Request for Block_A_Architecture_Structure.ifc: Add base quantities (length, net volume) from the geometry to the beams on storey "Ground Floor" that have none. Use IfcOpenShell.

First a look at what the model holds.

```python
import ifcopenshell
import ifcopenshell.util.element
import ifcopenshell.util.unit

model = ifcopenshell.open("Block_A_Architecture_Structure.ifc")
print(model.schema)
for unit_type in ("LENGTHUNIT", "AREAUNIT", "VOLUMEUNIT"):
    print(unit_type, ifcopenshell.util.unit.calculate_unit_scale(model, unit_type))
storey = next(s for s in model.by_type("IfcBuildingStorey") if s.Name == "Ground Floor")
beams = [e for e in ifcopenshell.util.element.get_decomposition(storey) if e.is_a("IfcBeam")]
for e in sorted(beams, key=lambda e: e.id()):
    print(e.id(), e.is_a(), e.Name, list(ifcopenshell.util.element.get_psets(e, qtos_only=True)), sep=" | ")
```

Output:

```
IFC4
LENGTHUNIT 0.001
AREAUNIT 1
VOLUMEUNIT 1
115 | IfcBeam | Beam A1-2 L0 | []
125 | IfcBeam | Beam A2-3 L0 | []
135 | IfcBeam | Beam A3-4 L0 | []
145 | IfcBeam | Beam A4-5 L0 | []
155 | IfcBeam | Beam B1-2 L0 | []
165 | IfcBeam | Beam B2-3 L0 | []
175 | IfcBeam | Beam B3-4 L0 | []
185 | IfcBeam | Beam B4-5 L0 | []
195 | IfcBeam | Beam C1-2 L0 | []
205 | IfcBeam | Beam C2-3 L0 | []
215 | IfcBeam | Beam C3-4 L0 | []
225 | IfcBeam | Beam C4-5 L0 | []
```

```python
import ifcopenshell
import ifcopenshell.api.pset
import ifcopenshell.geom
import ifcopenshell.util.element
import ifcopenshell.util.shape
import ifcopenshell.util.unit

model = ifcopenshell.open("Block_A_Architecture_Structure.ifc")
unit_scale = ifcopenshell.util.unit.calculate_unit_scale(model)
volume_scale = ifcopenshell.util.unit.calculate_unit_scale(model, "VOLUMEUNIT")
settings = ifcopenshell.geom.settings()

storey = next(s for s in model.by_type("IfcBuildingStorey") if s.Name == "Ground Floor")
beams = [e for e in ifcopenshell.util.element.get_decomposition(storey) if e.is_a("IfcBeam")]

for e in sorted(beams, key=lambda e: e.id()):
    if ifcopenshell.util.element.get_psets(e, qtos_only=True, should_inherit=False):
        continue
    # Geometry comes back in metres, in the element's own axes.
    shape = ifcopenshell.geom.create_shape(settings, e)
    values = {
        "Length": ifcopenshell.util.shape.get_max_xyz(shape.geometry) / unit_scale,
        "NetVolume": ifcopenshell.util.shape.get_volume(shape.geometry) / volume_scale,
    }
    qto = ifcopenshell.api.pset.add_qto(model, product=e, name="Qto_BeamBaseQuantities")
    ifcopenshell.api.pset.edit_qto(model, qto=qto, properties=values)
    print(e.id(), {k: round(v, 3) for k, v in values.items()})

model.write("Block_A_Architecture_Structure_rev.ifc")
```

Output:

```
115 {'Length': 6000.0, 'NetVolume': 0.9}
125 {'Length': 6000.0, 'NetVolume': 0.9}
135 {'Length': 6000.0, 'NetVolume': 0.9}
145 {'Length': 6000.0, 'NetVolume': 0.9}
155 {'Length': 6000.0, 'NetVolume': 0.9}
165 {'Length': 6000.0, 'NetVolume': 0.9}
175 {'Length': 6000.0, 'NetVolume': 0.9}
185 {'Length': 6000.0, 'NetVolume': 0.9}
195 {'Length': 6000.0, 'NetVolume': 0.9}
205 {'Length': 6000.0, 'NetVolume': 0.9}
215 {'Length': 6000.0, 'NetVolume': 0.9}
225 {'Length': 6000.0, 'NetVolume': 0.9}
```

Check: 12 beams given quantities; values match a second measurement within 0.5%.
